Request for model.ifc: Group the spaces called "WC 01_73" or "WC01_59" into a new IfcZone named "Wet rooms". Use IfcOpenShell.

First a look at what the model holds.

```python
import ifcopenshell

model = ifcopenshell.open("model.ifc")
print(model.schema)
seen = {}
for space in model.by_type("IfcSpace"):
    seen[space.Name] = seen.get(space.Name, 0) + 1
for name, count in sorted(seen.items(), key=str):
    print(count, "x", name)
print("zones:", [z.Name for z in model.by_type("IfcZone")][:20])
```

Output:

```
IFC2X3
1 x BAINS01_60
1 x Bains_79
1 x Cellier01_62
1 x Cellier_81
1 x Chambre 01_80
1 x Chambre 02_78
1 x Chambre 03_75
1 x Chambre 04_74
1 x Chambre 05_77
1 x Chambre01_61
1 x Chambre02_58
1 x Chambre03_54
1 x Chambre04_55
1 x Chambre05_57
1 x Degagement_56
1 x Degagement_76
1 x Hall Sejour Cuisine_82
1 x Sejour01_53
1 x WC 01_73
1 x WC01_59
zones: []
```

```python
import ifcopenshell
import ifcopenshell.api.group
import ifcopenshell.api.root

model = ifcopenshell.open("model.ifc")

names = {"WC 01_73", "WC01_59"}
spaces = [s for s in model.by_type("IfcSpace") if s.Name in names]

zone = ifcopenshell.api.root.create_entity(model, ifc_class="IfcZone", name="Wet rooms")
ifcopenshell.api.group.assign_group(model, products=spaces, group=zone)
print(len(spaces), "spaces in", zone.Name)

model.write("model_v2.ifc")
```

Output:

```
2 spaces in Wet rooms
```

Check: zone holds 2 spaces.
